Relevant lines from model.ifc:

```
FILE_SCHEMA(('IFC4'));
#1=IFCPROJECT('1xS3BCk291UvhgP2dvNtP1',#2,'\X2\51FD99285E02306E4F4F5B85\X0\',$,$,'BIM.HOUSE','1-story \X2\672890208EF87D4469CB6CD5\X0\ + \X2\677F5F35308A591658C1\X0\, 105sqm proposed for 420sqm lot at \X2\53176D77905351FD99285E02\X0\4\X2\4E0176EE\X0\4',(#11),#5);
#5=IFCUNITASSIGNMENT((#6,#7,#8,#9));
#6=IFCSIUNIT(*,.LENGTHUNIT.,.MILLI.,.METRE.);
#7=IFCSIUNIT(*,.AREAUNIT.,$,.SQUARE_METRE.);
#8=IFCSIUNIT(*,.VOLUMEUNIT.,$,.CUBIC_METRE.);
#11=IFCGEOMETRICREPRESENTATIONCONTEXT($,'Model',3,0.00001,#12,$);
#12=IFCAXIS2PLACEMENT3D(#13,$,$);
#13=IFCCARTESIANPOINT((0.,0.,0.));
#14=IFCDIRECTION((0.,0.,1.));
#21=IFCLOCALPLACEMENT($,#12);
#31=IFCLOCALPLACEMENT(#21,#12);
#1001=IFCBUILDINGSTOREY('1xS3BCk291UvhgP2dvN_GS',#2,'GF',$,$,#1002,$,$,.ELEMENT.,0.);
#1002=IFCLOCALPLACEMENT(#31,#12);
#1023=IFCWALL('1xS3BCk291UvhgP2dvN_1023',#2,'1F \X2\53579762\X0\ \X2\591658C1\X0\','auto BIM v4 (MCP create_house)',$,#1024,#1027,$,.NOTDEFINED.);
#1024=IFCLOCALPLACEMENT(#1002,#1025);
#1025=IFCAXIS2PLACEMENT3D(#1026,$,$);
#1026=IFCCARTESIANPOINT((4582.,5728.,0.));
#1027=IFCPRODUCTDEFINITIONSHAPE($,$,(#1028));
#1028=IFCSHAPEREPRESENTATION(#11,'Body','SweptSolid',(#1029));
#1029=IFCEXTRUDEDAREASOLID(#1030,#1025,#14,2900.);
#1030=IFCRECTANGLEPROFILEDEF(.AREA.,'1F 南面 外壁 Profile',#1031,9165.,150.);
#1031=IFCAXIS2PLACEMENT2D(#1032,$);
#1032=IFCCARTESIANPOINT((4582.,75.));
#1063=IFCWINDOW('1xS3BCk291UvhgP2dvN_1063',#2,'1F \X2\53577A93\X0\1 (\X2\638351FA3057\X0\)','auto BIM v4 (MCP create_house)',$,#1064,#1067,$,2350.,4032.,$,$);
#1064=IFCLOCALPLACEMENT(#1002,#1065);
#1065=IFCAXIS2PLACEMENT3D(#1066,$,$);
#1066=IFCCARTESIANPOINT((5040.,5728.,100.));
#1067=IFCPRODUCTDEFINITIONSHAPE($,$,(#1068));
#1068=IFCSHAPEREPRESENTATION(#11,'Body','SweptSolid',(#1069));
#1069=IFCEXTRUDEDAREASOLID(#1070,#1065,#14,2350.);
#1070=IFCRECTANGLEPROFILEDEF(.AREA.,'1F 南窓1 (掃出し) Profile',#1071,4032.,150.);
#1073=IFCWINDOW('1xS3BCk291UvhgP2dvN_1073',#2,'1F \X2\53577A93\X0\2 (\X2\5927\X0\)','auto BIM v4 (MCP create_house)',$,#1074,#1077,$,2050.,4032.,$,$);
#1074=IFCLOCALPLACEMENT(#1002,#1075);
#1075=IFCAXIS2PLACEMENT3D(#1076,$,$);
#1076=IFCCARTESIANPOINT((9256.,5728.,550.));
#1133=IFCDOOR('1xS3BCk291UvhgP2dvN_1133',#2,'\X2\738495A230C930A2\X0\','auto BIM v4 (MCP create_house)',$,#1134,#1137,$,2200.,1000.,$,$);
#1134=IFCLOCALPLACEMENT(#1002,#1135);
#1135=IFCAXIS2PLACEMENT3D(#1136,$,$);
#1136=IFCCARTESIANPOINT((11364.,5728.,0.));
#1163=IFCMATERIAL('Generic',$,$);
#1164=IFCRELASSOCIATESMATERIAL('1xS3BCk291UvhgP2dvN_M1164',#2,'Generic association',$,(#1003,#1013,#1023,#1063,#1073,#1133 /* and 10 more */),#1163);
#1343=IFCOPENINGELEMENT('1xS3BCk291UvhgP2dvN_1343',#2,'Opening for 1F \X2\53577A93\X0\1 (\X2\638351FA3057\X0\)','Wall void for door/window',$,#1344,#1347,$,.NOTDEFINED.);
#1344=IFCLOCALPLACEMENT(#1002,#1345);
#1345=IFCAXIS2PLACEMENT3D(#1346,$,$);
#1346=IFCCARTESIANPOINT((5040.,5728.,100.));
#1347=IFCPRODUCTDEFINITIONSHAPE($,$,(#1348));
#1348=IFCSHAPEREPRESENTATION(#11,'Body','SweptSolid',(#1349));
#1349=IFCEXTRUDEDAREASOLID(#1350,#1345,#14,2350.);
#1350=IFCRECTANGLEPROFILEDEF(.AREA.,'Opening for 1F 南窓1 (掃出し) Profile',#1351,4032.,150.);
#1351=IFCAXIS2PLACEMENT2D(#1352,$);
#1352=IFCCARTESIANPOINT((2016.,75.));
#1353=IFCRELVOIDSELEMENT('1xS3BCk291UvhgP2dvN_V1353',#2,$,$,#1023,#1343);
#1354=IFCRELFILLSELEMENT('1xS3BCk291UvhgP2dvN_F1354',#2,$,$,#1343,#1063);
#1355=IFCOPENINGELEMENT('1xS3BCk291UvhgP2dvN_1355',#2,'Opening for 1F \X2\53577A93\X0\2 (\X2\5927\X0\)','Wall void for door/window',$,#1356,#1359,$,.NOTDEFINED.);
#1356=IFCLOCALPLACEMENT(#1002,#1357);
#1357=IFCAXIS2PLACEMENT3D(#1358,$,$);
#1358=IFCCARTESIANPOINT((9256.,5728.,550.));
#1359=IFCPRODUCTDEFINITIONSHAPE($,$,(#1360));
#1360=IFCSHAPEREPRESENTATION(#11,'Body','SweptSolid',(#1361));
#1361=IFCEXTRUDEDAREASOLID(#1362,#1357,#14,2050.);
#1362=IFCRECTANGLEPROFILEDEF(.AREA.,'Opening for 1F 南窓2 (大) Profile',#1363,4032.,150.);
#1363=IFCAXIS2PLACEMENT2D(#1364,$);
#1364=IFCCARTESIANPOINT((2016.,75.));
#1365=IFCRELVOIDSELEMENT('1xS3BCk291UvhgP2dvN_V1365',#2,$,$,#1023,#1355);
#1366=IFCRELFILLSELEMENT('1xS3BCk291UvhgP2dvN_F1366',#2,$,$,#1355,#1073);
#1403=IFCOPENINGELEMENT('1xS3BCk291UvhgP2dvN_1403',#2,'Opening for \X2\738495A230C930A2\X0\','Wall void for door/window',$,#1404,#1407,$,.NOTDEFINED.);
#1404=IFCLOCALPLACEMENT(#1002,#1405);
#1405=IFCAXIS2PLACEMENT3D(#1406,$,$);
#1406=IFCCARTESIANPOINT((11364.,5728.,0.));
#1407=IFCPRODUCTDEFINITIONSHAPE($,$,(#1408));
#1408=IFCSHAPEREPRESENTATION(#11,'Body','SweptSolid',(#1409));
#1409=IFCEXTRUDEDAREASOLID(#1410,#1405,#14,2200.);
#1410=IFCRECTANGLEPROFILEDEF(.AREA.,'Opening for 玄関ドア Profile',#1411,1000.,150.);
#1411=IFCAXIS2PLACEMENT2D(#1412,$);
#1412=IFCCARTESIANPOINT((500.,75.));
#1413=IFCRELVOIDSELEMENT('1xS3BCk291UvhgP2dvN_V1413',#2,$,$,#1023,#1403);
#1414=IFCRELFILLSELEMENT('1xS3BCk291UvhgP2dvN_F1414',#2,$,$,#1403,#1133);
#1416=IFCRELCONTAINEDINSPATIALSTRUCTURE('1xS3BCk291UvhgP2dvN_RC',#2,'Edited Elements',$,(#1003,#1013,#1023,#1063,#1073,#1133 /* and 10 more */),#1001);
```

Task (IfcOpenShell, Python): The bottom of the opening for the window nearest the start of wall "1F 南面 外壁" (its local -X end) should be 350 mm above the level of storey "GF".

```python
import numpy as np
import ifcopenshell
import ifcopenshell.api.geometry
import ifcopenshell.geom
import ifcopenshell.util.element
import ifcopenshell.util.placement
import ifcopenshell.util.shape
import ifcopenshell.util.unit

model = ifcopenshell.open("model.ifc")
unit_scale = ifcopenshell.util.unit.calculate_unit_scale(model)

window = model.by_guid("1xS3BCk291UvhgP2dvN_1063")
opening = window.FillsVoids[0].RelatingOpeningElement
storey = ifcopenshell.util.element.get_container(window, ifc_class="IfcBuildingStorey")
level = ifcopenshell.util.placement.get_local_placement(storey.ObjectPlacement)[2, 3]

# The opening's origin need not be at the sill, so measure its lowest point.
shape = ifcopenshell.geom.create_shape(ifcopenshell.geom.settings(), opening)
bottom = ifcopenshell.util.shape.get_shape_bottom_elevation(shape, shape.geometry) / unit_scale
dz = level + 0.35 / unit_scale - bottom

shift = np.array([0.0, 0.0, dz])
# The window is not placed relative to its opening, so move both.
for product in (opening, window):
    matrix = ifcopenshell.util.placement.get_local_placement(product.ObjectPlacement)
    matrix[:3, 3] += shift
    ifcopenshell.api.geometry.edit_object_placement(model, product=product, matrix=matrix, is_si=False)

print(f"moved by {dz * unit_scale:+.3f} m")

model.write("model_updated.ifc")
```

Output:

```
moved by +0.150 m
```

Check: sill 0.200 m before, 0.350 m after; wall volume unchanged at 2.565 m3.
